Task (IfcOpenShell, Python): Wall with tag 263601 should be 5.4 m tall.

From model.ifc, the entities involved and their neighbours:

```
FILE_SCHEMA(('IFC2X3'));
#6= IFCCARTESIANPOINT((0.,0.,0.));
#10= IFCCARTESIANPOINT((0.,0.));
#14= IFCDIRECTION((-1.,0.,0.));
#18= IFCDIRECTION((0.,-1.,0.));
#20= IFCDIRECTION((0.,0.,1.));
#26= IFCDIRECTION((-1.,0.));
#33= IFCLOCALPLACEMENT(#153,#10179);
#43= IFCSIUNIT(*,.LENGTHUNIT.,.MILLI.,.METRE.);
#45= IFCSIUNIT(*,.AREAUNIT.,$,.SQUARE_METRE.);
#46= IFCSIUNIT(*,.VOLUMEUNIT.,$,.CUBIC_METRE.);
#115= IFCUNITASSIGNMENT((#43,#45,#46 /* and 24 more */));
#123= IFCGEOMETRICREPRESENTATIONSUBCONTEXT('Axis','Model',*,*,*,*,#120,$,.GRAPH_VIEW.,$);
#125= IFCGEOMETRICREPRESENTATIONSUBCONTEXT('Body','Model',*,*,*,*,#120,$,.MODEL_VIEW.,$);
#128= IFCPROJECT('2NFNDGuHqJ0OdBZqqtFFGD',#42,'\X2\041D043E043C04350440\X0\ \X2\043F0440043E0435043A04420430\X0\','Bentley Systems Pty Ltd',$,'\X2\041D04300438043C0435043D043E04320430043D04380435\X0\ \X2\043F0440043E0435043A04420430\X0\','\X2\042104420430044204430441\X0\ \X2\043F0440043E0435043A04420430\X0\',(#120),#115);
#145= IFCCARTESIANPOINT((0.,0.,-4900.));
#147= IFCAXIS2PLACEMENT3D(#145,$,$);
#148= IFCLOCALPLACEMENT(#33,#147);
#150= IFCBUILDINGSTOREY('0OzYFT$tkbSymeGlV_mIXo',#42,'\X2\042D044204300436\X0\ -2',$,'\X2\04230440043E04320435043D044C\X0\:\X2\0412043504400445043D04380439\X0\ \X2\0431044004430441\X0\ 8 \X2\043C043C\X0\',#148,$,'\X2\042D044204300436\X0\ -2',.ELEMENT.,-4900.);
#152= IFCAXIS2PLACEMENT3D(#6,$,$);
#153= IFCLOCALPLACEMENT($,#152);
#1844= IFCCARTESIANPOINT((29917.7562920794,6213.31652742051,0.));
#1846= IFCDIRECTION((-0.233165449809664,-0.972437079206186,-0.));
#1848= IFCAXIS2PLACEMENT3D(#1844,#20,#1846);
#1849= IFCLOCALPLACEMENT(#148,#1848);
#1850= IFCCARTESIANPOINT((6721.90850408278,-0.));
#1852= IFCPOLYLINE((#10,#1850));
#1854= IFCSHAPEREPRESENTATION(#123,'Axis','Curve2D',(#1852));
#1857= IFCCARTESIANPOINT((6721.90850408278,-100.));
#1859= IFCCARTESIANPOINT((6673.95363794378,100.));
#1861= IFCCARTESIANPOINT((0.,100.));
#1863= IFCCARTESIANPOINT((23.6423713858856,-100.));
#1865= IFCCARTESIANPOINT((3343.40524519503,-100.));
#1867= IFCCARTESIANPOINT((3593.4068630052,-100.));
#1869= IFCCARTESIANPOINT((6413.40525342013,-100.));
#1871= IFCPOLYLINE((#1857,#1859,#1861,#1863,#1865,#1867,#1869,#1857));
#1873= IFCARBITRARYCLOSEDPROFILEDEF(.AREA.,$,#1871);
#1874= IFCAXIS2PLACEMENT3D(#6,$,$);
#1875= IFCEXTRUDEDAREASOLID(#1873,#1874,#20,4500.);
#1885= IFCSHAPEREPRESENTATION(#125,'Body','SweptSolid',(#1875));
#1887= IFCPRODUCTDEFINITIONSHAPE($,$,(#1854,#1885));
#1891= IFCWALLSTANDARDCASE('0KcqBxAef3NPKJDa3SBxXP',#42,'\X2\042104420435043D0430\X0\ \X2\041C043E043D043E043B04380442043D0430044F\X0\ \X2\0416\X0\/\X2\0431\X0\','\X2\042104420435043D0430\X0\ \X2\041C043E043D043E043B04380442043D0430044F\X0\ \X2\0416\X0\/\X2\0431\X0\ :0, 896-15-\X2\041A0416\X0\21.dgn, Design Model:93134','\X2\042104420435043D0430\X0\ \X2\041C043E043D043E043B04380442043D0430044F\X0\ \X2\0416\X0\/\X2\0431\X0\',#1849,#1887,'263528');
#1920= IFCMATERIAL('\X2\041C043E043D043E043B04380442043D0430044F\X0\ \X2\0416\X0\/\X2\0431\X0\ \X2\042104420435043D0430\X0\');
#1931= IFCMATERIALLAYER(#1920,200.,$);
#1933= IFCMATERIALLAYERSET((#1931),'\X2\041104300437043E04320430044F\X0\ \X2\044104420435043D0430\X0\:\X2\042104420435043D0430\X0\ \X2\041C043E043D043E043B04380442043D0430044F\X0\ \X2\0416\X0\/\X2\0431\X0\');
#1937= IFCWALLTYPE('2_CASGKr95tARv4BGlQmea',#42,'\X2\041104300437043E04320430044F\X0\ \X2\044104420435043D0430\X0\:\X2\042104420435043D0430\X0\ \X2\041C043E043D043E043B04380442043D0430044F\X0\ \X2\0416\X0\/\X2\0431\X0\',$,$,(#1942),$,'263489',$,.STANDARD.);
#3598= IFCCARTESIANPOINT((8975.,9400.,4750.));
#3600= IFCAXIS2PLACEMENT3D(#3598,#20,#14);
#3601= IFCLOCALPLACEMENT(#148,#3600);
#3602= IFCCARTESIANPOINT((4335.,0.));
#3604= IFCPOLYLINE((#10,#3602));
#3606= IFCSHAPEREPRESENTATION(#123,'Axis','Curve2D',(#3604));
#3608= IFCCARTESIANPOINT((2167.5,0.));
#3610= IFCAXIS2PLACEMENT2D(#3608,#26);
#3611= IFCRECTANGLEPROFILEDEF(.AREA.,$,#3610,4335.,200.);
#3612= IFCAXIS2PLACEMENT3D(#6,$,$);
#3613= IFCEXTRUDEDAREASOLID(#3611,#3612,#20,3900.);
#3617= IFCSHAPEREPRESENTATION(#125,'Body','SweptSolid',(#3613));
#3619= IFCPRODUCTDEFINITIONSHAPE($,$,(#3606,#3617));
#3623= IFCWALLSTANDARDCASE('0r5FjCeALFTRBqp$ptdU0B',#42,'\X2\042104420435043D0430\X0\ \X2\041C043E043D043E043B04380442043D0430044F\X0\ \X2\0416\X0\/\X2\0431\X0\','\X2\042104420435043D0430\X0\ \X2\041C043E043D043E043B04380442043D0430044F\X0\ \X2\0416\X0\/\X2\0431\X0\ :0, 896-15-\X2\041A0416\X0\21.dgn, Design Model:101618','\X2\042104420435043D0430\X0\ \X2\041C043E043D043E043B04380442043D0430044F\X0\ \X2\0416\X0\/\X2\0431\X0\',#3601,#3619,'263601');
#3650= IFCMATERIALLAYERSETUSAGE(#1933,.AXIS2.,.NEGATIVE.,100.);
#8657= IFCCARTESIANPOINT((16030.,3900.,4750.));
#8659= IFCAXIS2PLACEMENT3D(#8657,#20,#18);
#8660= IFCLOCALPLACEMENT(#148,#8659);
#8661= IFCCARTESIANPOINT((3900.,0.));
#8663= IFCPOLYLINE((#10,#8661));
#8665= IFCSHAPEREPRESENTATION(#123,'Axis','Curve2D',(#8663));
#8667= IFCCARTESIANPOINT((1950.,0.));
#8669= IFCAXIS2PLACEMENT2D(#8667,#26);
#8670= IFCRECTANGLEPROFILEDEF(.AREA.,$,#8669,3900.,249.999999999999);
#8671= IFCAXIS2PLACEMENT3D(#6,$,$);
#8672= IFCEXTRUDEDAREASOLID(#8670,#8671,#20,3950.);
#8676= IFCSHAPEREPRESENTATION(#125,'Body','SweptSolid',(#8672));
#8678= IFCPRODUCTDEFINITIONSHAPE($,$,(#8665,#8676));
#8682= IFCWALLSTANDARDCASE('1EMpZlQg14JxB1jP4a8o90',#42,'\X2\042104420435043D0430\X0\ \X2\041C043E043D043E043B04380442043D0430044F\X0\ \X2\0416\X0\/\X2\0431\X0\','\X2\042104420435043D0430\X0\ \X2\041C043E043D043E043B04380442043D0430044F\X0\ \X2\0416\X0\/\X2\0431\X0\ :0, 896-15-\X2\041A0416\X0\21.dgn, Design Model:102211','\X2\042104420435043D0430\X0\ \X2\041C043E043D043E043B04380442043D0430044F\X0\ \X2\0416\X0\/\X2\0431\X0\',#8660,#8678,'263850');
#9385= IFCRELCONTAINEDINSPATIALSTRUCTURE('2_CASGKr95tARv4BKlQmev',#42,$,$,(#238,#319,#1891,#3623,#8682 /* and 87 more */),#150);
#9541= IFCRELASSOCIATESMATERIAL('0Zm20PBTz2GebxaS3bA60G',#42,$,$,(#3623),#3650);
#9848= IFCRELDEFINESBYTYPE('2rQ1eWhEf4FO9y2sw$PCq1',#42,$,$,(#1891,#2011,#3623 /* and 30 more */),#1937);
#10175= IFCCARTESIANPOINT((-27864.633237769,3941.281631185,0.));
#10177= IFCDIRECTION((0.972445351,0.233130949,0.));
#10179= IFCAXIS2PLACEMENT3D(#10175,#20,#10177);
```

```python
import ifcopenshell
import ifcopenshell.geom
import ifcopenshell.util.representation
import ifcopenshell.util.shape
import ifcopenshell.util.unit

model = ifcopenshell.open("model.ifc")
unit_scale = ifcopenshell.util.unit.calculate_unit_scale(model)
settings = ifcopenshell.geom.settings()


def volume(element):
    """Net volume in cubic metres, openings subtracted."""
    shape = ifcopenshell.geom.create_shape(settings, element)
    return ifcopenshell.util.shape.get_volume(shape.geometry)


wall = model.by_guid("0r5FjCeALFTRBqp$ptdU0B")
before = volume(wall)

body = ifcopenshell.util.representation.get_representation(wall, "Model", "Body")
solid = body.Items[0]
old_height = solid.Depth
solid.Depth = 5.4 / unit_scale
after = volume(wall)

print(f"height {old_height:g} -> {solid.Depth:g}, volume {before:.3f} -> {after:.3f} m3")

model.write("model_v2.ifc")
```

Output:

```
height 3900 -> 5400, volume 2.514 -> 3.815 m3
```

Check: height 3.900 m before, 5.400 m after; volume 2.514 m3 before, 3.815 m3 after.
